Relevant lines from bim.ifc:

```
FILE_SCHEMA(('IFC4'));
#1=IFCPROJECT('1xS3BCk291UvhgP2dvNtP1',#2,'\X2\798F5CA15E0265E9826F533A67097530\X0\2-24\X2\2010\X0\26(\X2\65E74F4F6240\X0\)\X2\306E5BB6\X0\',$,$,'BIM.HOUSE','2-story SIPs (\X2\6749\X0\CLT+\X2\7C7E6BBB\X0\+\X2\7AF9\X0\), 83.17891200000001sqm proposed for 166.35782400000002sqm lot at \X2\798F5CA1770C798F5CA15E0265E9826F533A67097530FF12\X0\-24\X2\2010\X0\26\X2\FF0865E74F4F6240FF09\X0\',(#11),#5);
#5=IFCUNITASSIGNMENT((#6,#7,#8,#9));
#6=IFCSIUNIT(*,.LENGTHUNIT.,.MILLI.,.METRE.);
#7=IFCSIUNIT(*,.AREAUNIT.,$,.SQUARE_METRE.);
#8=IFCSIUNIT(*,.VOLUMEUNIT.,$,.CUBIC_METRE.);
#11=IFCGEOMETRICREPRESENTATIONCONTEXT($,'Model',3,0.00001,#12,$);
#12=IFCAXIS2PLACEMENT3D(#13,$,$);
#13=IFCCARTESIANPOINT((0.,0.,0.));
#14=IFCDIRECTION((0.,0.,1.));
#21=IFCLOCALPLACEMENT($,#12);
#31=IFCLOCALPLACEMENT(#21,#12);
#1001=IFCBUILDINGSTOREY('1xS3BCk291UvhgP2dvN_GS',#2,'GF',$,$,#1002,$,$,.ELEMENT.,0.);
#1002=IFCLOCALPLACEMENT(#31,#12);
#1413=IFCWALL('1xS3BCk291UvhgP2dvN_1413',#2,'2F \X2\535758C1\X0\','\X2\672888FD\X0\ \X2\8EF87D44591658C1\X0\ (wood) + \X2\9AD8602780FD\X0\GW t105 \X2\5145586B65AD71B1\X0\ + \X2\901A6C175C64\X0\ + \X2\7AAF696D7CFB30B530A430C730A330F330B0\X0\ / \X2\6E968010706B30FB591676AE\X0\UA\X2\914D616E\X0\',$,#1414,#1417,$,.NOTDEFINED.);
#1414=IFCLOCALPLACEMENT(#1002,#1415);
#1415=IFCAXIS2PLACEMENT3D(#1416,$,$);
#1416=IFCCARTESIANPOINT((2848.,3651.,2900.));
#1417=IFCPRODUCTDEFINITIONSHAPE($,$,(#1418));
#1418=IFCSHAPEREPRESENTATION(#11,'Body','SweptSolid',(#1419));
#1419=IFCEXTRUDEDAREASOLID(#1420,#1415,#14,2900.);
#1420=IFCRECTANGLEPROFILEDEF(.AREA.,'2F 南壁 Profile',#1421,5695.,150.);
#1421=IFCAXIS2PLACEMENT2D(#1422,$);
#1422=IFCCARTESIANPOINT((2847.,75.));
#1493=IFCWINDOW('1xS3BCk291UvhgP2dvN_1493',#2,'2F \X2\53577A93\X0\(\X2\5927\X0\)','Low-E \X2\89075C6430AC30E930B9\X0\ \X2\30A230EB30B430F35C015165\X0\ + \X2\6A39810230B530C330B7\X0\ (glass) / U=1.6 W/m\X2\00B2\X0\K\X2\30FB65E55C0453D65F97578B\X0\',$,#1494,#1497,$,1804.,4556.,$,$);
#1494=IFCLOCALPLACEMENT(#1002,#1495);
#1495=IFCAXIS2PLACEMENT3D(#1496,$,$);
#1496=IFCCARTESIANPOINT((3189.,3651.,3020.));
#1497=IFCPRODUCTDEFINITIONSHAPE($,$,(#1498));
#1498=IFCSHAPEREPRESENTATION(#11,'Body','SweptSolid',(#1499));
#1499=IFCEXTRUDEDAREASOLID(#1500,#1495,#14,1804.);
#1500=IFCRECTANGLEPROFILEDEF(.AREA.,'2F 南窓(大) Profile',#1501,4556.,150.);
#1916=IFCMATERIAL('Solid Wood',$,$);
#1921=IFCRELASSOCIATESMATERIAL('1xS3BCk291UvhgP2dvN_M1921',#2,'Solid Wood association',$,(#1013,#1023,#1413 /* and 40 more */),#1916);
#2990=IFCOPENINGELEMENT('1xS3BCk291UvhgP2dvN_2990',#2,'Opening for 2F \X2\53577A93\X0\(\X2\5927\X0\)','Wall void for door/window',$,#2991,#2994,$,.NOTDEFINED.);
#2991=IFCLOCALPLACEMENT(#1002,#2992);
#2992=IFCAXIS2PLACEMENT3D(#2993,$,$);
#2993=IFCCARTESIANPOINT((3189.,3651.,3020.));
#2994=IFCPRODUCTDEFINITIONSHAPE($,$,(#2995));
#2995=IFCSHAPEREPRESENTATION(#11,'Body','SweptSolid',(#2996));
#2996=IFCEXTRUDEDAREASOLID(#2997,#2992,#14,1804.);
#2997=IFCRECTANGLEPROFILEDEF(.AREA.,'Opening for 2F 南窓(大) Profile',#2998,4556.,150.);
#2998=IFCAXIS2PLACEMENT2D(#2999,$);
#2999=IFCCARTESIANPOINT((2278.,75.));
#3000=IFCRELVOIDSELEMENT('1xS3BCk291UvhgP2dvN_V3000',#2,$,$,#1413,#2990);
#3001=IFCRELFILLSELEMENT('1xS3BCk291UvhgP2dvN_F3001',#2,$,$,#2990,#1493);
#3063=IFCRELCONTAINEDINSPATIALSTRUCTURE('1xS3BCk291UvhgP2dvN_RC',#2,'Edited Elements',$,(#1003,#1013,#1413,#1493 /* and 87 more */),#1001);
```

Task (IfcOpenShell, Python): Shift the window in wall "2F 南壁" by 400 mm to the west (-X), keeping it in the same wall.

```python
import ifcopenshell
import ifcopenshell.api.geometry
import ifcopenshell.util.placement

model = ifcopenshell.open("bim.ifc")

window = model.by_guid("1xS3BCk291UvhgP2dvN_1493")
opening = window.FillsVoids[0].RelatingOpeningElement
wall = opening.VoidsElements[0].RelatingBuildingElement

wall_matrix = ifcopenshell.util.placement.get_local_placement(wall.ObjectPlacement)
shift = wall_matrix[:3, 0] * -400.0
before = ifcopenshell.util.placement.get_local_placement(window.ObjectPlacement)[:3, 3].copy()

# The window is not placed relative to its opening, so move both.
for product in (opening, window):
    matrix = ifcopenshell.util.placement.get_local_placement(product.ObjectPlacement)
    matrix[:3, 3] += shift
    ifcopenshell.api.geometry.edit_object_placement(model, product=product, matrix=matrix, is_si=False)

after = ifcopenshell.util.placement.get_local_placement(window.ObjectPlacement)[:3, 3]
print("window moved by", (after - before).round(3) + 0.0)

model.write("bim-out.ifc")
```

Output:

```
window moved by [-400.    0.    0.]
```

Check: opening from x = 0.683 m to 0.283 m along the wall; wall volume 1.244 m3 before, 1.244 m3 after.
